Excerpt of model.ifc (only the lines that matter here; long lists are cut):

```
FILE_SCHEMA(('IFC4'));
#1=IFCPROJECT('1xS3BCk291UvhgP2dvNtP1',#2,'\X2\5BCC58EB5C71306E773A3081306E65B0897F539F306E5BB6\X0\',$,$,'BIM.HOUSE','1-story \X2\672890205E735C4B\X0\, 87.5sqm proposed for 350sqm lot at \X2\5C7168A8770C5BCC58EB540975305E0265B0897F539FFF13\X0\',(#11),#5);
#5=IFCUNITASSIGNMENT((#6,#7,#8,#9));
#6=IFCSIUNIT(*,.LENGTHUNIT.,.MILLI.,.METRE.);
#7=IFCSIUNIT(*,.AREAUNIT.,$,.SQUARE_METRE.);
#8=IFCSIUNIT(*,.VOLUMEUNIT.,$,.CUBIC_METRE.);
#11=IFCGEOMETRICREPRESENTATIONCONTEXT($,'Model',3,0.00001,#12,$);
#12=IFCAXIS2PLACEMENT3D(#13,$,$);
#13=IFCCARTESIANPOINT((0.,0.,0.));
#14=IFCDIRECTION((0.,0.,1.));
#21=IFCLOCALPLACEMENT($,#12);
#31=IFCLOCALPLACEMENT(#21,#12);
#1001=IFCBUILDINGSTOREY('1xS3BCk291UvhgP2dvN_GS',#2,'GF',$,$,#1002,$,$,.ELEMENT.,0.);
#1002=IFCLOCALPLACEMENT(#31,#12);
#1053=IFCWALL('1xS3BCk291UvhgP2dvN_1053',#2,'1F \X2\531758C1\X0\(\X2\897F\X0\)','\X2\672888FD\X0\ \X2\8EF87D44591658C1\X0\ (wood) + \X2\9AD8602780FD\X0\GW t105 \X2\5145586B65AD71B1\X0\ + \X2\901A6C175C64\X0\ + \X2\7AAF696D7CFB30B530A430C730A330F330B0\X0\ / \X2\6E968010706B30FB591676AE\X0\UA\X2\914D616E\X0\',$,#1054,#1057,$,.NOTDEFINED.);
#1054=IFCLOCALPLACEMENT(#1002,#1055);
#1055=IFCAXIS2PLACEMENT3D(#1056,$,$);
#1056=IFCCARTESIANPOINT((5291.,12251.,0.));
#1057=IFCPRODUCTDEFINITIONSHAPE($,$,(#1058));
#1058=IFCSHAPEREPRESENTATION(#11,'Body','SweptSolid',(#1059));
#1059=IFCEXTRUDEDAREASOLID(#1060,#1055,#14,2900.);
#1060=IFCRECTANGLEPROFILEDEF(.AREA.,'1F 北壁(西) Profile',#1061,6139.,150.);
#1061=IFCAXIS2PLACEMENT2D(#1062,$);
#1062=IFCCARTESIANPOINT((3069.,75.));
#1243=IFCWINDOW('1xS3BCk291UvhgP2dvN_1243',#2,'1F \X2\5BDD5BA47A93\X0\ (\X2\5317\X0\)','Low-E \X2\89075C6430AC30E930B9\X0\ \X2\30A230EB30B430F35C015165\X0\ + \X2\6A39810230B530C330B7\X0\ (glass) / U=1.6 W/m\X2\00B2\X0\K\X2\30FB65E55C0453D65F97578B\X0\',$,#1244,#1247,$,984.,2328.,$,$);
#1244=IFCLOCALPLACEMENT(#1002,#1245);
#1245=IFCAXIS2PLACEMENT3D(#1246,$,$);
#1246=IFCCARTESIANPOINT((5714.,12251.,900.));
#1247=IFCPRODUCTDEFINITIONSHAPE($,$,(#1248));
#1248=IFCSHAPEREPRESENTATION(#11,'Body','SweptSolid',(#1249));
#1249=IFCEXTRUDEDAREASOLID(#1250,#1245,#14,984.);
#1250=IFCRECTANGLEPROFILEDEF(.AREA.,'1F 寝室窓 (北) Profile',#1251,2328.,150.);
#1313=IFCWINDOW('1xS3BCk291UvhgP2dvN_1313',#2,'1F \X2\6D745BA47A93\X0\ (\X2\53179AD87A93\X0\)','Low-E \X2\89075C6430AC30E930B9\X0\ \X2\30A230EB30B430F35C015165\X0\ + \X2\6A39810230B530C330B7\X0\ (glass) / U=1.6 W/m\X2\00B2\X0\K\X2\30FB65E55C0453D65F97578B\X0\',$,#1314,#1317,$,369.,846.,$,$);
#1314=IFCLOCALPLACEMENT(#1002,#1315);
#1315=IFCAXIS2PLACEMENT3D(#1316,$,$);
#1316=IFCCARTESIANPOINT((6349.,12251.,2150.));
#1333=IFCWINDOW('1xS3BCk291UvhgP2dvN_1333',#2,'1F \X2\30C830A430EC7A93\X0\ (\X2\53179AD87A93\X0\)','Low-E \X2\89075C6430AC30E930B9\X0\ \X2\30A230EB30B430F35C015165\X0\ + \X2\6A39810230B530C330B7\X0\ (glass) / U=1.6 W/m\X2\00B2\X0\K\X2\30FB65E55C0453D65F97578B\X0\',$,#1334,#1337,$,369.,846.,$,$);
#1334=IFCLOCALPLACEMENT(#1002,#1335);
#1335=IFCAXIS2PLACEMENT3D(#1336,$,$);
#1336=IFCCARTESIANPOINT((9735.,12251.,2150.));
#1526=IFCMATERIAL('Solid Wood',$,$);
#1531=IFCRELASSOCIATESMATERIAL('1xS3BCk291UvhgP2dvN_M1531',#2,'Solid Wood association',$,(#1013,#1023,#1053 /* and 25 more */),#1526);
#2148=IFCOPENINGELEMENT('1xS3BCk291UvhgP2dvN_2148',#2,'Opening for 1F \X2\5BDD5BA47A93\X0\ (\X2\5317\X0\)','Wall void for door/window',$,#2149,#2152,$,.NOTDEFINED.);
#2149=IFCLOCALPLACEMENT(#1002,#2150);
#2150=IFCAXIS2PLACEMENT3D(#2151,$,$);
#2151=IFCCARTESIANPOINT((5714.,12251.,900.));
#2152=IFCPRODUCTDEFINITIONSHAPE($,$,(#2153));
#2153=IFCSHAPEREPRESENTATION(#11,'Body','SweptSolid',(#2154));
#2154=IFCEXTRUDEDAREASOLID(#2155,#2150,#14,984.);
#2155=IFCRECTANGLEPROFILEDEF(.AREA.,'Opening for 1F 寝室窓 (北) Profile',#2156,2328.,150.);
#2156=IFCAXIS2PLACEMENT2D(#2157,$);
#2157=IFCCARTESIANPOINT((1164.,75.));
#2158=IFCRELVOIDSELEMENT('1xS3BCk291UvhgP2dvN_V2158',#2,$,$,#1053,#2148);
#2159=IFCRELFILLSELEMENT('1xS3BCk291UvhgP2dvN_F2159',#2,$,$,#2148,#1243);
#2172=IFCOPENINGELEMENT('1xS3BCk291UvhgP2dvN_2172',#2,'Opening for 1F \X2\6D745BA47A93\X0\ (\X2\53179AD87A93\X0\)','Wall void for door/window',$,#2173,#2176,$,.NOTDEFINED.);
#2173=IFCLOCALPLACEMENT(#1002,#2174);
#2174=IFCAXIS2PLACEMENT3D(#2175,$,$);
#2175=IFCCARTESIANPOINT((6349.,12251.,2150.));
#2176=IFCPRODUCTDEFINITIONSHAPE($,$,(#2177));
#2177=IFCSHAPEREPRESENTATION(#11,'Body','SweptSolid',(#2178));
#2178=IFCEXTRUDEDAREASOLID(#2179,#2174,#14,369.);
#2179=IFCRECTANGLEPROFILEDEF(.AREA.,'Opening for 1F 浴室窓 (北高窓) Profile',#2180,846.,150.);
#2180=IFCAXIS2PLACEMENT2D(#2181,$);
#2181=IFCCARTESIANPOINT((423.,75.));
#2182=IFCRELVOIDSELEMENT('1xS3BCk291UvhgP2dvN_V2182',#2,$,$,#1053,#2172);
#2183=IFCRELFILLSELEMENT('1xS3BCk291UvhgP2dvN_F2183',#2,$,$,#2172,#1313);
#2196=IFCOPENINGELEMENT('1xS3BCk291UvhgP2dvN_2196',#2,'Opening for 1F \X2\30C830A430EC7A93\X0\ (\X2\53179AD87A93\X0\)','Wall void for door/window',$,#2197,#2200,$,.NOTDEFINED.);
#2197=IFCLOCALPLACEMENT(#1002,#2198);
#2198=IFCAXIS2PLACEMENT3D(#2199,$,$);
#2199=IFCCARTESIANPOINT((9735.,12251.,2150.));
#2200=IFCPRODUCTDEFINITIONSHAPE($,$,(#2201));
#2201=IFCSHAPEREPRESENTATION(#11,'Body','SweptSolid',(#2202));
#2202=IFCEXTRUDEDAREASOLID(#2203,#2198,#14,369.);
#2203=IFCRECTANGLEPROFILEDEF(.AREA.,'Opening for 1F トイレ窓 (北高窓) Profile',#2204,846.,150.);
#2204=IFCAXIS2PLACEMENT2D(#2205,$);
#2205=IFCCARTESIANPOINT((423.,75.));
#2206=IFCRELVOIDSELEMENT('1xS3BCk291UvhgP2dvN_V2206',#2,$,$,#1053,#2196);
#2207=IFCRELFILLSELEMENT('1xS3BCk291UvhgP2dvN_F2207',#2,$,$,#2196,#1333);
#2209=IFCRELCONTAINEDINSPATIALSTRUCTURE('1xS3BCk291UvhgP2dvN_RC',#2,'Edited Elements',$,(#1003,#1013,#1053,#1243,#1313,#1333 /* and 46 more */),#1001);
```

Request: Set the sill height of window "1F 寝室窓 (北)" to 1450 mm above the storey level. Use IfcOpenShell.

```python
import numpy as np
import ifcopenshell
import ifcopenshell.api.geometry
import ifcopenshell.geom
import ifcopenshell.util.element
import ifcopenshell.util.placement
import ifcopenshell.util.shape
import ifcopenshell.util.unit

model = ifcopenshell.open("model.ifc")
unit_scale = ifcopenshell.util.unit.calculate_unit_scale(model)

window = model.by_guid("1xS3BCk291UvhgP2dvN_1243")
opening = window.FillsVoids[0].RelatingOpeningElement
storey = ifcopenshell.util.element.get_container(window, ifc_class="IfcBuildingStorey")
level = ifcopenshell.util.placement.get_local_placement(storey.ObjectPlacement)[2, 3]

# The opening's origin need not be at the sill, so measure its lowest point.
shape = ifcopenshell.geom.create_shape(ifcopenshell.geom.settings(), opening)
bottom = ifcopenshell.util.shape.get_shape_bottom_elevation(shape, shape.geometry) / unit_scale
dz = level + 1450.0 - bottom

shift = np.array([0.0, 0.0, dz])
# The window is not placed relative to its opening, so move both.
for product in (opening, window):
    matrix = ifcopenshell.util.placement.get_local_placement(product.ObjectPlacement)
    matrix[:3, 3] += shift
    ifcopenshell.api.geometry.edit_object_placement(model, product=product, matrix=matrix, is_si=False)

print(f"moved by {dz * unit_scale:+.3f} m")

model.write("model_edited.ifc")
```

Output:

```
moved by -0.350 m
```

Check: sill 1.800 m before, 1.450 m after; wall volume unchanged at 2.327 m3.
